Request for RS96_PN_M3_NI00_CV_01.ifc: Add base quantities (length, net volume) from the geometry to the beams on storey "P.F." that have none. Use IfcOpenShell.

First a look at what the model holds.

```python
import ifcopenshell
import ifcopenshell.util.element
import ifcopenshell.util.unit

model = ifcopenshell.open("RS96_PN_M3_NI00_CV_01.ifc")
print(model.schema)
for unit_type in ("LENGTHUNIT", "AREAUNIT", "VOLUMEUNIT"):
    print(unit_type, ifcopenshell.util.unit.calculate_unit_scale(model, unit_type))
storey = next(s for s in model.by_type("IfcBuildingStorey") if s.Name == "P.F.")
beams = [e for e in ifcopenshell.util.element.get_decomposition(storey) if e.is_a("IfcBeam")]
for e in sorted(beams, key=lambda e: e.id()):
    print(e.id(), e.is_a(), e.Name, list(ifcopenshell.util.element.get_psets(e, qtos_only=True)), sep=" | ")
```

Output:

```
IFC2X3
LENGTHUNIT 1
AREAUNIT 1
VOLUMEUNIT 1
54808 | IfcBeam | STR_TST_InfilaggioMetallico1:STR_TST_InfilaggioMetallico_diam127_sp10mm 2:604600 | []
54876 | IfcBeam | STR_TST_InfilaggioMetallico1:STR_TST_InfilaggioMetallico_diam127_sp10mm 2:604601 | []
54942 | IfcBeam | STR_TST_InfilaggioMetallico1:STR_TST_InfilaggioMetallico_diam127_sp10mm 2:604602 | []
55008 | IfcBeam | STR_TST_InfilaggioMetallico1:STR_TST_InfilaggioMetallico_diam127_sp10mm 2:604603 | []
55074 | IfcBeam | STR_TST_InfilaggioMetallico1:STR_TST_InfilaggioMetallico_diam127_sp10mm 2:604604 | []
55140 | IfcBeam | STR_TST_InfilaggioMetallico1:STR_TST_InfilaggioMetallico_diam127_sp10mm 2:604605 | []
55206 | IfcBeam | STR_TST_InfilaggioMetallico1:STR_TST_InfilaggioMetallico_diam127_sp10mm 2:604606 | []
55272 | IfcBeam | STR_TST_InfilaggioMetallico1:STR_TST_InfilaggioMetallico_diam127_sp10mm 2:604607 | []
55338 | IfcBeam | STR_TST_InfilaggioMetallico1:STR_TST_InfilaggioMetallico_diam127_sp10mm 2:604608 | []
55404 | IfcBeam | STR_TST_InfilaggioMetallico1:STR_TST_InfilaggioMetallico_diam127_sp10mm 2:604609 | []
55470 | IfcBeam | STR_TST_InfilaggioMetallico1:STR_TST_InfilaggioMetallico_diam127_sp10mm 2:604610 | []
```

```python
import ifcopenshell
import ifcopenshell.api.pset
import ifcopenshell.geom
import ifcopenshell.util.element
import ifcopenshell.util.shape
import ifcopenshell.util.unit

model = ifcopenshell.open("RS96_PN_M3_NI00_CV_01.ifc")
unit_scale = ifcopenshell.util.unit.calculate_unit_scale(model)
volume_scale = ifcopenshell.util.unit.calculate_unit_scale(model, "VOLUMEUNIT")
settings = ifcopenshell.geom.settings()

storey = next(s for s in model.by_type("IfcBuildingStorey") if s.Name == "P.F.")
beams = [e for e in ifcopenshell.util.element.get_decomposition(storey) if e.is_a("IfcBeam")]

for e in sorted(beams, key=lambda e: e.id()):
    if ifcopenshell.util.element.get_psets(e, qtos_only=True, should_inherit=False):
        continue
    # Geometry comes back in metres, in the element's own axes.
    shape = ifcopenshell.geom.create_shape(settings, e)
    values = {
        "Length": ifcopenshell.util.shape.get_max_xyz(shape.geometry) / unit_scale,
        "NetVolume": ifcopenshell.util.shape.get_volume(shape.geometry) / volume_scale,
    }
    qto = ifcopenshell.api.pset.add_qto(model, product=e, name="BaseQuantities")
    ifcopenshell.api.pset.edit_qto(model, qto=qto, properties=values)
    print(e.id(), {k: round(v, 3) for k, v in values.items()})

model.write("RS96_PN_M3_NI00_CV_01_v2.ifc")
```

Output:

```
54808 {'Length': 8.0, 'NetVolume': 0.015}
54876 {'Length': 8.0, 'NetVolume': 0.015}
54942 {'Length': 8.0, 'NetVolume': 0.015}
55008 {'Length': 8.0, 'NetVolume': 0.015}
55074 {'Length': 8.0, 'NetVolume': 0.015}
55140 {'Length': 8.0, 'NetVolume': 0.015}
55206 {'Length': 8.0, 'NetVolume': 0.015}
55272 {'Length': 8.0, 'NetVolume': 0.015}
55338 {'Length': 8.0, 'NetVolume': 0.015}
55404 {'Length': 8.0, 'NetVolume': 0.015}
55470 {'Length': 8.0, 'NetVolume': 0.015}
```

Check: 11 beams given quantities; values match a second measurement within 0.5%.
